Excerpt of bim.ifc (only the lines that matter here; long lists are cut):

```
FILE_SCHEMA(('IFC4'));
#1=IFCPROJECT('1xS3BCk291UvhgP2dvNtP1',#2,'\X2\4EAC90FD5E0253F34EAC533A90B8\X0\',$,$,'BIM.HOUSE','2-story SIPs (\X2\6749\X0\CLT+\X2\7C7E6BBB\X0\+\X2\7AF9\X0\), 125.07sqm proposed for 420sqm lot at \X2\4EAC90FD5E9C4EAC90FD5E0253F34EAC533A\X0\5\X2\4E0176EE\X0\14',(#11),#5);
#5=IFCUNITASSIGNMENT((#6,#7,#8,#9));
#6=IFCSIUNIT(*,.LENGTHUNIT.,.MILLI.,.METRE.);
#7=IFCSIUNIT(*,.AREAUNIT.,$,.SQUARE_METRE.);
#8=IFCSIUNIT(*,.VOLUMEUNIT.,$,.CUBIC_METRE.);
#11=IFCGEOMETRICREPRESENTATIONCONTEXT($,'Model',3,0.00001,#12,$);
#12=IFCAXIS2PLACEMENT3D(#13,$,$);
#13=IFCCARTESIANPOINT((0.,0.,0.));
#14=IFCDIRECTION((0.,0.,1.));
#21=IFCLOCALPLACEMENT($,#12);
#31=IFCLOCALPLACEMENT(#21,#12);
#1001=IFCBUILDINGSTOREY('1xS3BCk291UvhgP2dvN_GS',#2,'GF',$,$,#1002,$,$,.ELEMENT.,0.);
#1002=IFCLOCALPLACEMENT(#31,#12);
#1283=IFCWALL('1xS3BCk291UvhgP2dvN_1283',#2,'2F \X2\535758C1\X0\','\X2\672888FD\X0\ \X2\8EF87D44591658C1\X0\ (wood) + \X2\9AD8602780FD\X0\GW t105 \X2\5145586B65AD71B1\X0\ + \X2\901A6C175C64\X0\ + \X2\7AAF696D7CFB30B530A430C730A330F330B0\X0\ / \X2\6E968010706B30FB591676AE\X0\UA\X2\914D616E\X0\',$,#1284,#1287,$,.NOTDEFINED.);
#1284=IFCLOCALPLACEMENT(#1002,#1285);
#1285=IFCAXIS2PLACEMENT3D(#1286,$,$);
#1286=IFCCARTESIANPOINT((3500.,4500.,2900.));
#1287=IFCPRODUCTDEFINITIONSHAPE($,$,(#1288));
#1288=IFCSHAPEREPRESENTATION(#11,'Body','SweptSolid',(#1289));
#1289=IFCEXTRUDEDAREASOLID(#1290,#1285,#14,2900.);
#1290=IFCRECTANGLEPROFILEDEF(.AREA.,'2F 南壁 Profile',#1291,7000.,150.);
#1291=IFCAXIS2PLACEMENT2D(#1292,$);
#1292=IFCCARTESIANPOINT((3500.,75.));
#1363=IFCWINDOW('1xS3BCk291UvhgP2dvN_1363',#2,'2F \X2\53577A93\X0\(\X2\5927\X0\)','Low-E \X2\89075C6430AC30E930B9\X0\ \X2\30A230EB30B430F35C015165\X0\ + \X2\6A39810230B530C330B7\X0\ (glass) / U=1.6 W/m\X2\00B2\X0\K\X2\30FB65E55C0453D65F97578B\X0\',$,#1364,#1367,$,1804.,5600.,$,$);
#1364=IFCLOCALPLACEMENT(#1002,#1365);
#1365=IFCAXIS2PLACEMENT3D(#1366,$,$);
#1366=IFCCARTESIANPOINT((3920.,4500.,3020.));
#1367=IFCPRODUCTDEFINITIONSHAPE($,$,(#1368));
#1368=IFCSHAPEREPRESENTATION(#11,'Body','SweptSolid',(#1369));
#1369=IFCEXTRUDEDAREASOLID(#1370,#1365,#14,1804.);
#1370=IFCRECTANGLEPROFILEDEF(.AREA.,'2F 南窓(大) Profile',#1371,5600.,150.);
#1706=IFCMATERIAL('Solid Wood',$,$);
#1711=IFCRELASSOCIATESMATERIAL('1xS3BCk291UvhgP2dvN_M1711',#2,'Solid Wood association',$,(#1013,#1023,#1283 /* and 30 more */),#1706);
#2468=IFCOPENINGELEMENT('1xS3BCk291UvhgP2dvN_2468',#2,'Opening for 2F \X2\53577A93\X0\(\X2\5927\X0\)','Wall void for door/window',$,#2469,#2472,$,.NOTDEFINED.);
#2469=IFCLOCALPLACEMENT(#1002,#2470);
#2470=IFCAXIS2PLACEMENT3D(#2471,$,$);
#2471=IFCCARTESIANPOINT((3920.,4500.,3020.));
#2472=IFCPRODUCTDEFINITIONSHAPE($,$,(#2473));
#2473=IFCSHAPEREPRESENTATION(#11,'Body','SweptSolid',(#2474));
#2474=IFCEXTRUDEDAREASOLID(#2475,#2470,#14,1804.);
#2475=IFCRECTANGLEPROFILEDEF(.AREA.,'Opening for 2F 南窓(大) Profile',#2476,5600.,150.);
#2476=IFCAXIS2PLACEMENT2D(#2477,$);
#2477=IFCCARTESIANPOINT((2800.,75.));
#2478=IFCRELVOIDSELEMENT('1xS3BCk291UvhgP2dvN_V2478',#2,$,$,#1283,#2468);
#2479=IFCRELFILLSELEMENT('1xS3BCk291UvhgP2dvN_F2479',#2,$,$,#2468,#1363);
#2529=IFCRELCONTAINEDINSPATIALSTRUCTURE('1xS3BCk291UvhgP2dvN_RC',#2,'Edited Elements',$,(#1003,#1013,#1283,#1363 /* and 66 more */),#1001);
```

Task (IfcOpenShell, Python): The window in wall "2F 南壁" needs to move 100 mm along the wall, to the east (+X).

```python
import ifcopenshell
import ifcopenshell.api.geometry
import ifcopenshell.util.placement
import ifcopenshell.util.unit

model = ifcopenshell.open("bim.ifc")
unit_scale = ifcopenshell.util.unit.calculate_unit_scale(model)

window = model.by_guid("1xS3BCk291UvhgP2dvN_1363")
opening = window.FillsVoids[0].RelatingOpeningElement
wall = opening.VoidsElements[0].RelatingBuildingElement

wall_matrix = ifcopenshell.util.placement.get_local_placement(wall.ObjectPlacement)
shift = wall_matrix[:3, 0] * 0.1 / unit_scale
before = ifcopenshell.util.placement.get_local_placement(window.ObjectPlacement)[:3, 3].copy()

# The window is not placed relative to its opening, so move both.
for product in (opening, window):
    matrix = ifcopenshell.util.placement.get_local_placement(product.ObjectPlacement)
    matrix[:3, 3] += shift
    ifcopenshell.api.geometry.edit_object_placement(model, product=product, matrix=matrix, is_si=False)

after = ifcopenshell.util.placement.get_local_placement(window.ObjectPlacement)[:3, 3]
print("window moved by", (after - before).round(3) + 0.0)

model.write("bim_v2.ifc")
```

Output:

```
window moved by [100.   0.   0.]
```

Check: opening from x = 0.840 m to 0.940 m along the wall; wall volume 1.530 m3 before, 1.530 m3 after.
